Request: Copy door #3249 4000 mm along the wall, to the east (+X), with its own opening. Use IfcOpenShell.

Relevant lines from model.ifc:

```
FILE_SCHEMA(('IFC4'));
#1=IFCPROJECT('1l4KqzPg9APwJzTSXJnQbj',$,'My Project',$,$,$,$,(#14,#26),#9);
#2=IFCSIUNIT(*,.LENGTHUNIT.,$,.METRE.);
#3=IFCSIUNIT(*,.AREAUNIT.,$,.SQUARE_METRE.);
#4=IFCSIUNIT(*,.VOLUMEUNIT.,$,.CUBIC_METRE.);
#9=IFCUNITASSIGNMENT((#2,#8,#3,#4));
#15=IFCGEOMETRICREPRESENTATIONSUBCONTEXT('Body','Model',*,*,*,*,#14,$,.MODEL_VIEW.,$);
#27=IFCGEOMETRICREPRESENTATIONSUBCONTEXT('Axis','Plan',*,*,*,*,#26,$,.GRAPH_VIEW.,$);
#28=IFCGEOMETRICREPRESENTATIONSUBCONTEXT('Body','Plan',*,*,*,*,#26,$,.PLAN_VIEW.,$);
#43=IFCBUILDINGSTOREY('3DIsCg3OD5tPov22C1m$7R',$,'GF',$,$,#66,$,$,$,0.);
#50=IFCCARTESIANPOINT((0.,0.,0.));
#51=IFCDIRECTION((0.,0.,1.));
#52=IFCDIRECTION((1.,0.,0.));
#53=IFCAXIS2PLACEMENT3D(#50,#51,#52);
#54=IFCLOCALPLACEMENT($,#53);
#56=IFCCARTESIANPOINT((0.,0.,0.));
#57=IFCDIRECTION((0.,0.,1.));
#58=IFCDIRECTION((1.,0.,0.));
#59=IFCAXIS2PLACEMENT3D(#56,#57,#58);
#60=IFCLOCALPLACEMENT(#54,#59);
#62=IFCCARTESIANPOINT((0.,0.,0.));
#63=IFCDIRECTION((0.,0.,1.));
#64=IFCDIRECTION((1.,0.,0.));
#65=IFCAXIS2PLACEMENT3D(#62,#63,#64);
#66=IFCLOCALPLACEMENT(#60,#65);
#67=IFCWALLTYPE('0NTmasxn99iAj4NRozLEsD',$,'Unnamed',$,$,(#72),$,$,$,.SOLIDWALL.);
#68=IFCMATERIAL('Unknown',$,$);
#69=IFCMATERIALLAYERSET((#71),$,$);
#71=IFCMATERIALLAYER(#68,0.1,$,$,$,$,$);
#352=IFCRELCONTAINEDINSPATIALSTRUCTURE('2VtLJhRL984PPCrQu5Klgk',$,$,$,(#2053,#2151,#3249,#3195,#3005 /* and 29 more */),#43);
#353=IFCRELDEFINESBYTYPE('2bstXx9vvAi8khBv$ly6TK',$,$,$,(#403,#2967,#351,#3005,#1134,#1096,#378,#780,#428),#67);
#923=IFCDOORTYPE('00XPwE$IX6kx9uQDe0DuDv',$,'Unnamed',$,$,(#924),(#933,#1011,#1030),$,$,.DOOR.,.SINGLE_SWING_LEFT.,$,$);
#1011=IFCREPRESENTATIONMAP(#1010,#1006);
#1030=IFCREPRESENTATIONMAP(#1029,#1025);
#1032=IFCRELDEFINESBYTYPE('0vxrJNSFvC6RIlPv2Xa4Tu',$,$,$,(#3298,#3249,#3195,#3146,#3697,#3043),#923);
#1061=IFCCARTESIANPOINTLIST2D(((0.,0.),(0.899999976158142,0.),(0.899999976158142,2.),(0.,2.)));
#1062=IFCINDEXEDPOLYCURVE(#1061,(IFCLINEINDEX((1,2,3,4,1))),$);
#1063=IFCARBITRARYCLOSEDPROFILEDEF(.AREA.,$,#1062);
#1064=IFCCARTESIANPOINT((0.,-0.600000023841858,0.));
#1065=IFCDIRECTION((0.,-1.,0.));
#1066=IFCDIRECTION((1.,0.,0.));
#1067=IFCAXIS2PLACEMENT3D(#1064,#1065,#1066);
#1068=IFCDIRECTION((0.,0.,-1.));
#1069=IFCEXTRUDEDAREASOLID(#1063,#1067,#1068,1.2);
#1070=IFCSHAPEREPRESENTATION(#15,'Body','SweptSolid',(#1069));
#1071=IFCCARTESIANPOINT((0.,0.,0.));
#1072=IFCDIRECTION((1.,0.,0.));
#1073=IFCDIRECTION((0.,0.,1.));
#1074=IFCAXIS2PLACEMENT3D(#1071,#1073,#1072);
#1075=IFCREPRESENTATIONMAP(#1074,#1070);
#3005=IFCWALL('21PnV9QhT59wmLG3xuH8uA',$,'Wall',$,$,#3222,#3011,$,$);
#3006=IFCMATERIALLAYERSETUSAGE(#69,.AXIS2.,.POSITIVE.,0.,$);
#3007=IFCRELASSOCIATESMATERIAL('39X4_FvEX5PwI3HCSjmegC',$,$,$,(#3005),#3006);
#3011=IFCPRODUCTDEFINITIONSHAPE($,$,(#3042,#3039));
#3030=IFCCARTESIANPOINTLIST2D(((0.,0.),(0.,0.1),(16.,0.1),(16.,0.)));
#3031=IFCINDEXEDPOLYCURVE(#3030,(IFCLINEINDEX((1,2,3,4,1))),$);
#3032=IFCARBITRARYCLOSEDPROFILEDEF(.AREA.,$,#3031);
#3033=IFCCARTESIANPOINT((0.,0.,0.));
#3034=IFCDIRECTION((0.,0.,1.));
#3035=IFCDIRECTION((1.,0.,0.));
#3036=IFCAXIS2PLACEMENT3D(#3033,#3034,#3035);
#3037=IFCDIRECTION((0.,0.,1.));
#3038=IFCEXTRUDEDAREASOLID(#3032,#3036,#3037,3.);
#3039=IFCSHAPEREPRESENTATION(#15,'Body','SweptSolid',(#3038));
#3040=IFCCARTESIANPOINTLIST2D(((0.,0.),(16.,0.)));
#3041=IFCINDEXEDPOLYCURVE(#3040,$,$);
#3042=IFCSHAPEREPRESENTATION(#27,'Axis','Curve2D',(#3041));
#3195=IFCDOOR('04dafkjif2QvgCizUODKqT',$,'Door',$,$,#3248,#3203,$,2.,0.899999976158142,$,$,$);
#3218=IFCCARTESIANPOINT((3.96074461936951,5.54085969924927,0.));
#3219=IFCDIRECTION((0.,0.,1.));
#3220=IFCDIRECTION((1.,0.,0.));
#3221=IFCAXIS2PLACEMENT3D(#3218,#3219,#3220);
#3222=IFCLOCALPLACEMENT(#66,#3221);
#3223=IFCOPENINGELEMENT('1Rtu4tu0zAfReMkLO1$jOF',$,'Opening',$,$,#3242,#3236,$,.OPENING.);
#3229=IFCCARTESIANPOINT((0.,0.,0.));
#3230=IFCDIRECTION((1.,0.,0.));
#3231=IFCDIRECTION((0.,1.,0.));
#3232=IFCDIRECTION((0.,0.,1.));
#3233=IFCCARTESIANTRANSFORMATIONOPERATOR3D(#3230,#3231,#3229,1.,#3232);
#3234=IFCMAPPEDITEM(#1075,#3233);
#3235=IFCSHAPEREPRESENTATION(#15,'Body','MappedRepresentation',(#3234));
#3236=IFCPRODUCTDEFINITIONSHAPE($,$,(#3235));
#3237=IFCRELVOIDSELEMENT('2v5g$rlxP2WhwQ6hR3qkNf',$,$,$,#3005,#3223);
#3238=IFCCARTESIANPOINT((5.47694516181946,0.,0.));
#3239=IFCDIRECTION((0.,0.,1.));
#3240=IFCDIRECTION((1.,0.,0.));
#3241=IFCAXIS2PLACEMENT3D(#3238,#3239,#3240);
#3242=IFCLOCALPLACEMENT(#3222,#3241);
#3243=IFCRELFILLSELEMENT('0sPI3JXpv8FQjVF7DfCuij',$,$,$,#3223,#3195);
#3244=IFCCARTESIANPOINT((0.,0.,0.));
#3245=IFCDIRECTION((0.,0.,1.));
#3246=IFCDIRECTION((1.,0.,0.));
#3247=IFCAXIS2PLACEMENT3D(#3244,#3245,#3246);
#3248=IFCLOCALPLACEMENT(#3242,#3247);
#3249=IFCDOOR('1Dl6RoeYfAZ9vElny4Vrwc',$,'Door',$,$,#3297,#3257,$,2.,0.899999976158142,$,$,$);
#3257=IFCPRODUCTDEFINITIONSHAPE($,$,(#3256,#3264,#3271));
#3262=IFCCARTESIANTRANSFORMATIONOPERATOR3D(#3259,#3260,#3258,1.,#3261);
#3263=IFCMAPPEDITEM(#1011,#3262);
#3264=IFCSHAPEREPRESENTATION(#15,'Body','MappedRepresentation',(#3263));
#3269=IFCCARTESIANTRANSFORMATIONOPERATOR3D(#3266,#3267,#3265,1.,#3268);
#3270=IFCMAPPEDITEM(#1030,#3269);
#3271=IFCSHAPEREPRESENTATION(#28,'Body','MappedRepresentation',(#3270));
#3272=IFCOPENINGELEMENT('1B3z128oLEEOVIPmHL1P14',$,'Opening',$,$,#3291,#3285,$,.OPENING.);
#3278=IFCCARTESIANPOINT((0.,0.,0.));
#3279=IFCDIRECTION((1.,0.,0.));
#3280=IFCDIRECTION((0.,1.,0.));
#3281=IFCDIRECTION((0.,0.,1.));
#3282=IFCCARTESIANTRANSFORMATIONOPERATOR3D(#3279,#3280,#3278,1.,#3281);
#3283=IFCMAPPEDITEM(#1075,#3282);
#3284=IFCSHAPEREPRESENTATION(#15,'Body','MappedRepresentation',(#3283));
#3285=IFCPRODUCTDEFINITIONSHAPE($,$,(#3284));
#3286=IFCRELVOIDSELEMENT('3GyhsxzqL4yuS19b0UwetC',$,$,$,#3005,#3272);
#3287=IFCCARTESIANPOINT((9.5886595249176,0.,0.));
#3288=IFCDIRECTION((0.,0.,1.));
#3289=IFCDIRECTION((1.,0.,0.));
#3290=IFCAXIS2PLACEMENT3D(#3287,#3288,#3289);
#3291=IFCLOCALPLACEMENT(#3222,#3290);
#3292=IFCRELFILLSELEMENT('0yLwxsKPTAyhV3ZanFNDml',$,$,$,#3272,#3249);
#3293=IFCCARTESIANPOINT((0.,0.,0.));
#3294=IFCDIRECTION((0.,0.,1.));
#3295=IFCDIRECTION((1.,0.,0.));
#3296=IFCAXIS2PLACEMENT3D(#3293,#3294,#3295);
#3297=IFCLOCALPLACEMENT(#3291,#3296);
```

```python
import ifcopenshell
import ifcopenshell.api.feature
import ifcopenshell.api.geometry
import ifcopenshell.api.root
import ifcopenshell.geom
import ifcopenshell.util.element
import ifcopenshell.util.placement
import ifcopenshell.util.shape

model = ifcopenshell.open("model.ifc")
settings = ifcopenshell.geom.settings()


def volume(element):
    """Net volume in cubic metres, openings subtracted."""
    shape = ifcopenshell.geom.create_shape(settings, element)
    return ifcopenshell.util.shape.get_volume(shape.geometry)


door = model.by_guid("1Dl6RoeYfAZ9vElny4Vrwc")
opening = door.FillsVoids[0].RelatingOpeningElement
wall = opening.VoidsElements[0].RelatingBuildingElement
before = volume(wall)
shift = ifcopenshell.util.placement.get_local_placement(wall.ObjectPlacement)[:3, 0] * 4.0

# copy_class copies the void relationship, type, container and properties, but no geometry.
new_opening = ifcopenshell.api.root.copy_class(model, product=opening)
new_opening.Representation = ifcopenshell.util.element.copy_deep(
    model, opening.Representation, exclude=["IfcGeometricRepresentationContext", "IfcRepresentationMap"]
)
new_door = ifcopenshell.api.root.copy_class(model, product=door)
new_door.Representation = ifcopenshell.util.element.copy_deep(
    model, door.Representation, exclude=["IfcGeometricRepresentationContext", "IfcRepresentationMap"]
)
ifcopenshell.api.feature.add_filling(model, opening=new_opening, element=new_door)

for old, new in ((opening, new_opening), (door, new_door)):
    matrix = ifcopenshell.util.placement.get_local_placement(old.ObjectPlacement)
    matrix[:3, 3] += shift
    ifcopenshell.api.geometry.edit_object_placement(model, product=new, matrix=matrix, is_si=False)

after = volume(wall)

print(f"wall volume {before:.3f} -> {after:.3f} m3")

model.write("model-out.ifc")
```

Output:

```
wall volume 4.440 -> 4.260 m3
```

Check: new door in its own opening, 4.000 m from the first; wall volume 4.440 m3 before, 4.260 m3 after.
